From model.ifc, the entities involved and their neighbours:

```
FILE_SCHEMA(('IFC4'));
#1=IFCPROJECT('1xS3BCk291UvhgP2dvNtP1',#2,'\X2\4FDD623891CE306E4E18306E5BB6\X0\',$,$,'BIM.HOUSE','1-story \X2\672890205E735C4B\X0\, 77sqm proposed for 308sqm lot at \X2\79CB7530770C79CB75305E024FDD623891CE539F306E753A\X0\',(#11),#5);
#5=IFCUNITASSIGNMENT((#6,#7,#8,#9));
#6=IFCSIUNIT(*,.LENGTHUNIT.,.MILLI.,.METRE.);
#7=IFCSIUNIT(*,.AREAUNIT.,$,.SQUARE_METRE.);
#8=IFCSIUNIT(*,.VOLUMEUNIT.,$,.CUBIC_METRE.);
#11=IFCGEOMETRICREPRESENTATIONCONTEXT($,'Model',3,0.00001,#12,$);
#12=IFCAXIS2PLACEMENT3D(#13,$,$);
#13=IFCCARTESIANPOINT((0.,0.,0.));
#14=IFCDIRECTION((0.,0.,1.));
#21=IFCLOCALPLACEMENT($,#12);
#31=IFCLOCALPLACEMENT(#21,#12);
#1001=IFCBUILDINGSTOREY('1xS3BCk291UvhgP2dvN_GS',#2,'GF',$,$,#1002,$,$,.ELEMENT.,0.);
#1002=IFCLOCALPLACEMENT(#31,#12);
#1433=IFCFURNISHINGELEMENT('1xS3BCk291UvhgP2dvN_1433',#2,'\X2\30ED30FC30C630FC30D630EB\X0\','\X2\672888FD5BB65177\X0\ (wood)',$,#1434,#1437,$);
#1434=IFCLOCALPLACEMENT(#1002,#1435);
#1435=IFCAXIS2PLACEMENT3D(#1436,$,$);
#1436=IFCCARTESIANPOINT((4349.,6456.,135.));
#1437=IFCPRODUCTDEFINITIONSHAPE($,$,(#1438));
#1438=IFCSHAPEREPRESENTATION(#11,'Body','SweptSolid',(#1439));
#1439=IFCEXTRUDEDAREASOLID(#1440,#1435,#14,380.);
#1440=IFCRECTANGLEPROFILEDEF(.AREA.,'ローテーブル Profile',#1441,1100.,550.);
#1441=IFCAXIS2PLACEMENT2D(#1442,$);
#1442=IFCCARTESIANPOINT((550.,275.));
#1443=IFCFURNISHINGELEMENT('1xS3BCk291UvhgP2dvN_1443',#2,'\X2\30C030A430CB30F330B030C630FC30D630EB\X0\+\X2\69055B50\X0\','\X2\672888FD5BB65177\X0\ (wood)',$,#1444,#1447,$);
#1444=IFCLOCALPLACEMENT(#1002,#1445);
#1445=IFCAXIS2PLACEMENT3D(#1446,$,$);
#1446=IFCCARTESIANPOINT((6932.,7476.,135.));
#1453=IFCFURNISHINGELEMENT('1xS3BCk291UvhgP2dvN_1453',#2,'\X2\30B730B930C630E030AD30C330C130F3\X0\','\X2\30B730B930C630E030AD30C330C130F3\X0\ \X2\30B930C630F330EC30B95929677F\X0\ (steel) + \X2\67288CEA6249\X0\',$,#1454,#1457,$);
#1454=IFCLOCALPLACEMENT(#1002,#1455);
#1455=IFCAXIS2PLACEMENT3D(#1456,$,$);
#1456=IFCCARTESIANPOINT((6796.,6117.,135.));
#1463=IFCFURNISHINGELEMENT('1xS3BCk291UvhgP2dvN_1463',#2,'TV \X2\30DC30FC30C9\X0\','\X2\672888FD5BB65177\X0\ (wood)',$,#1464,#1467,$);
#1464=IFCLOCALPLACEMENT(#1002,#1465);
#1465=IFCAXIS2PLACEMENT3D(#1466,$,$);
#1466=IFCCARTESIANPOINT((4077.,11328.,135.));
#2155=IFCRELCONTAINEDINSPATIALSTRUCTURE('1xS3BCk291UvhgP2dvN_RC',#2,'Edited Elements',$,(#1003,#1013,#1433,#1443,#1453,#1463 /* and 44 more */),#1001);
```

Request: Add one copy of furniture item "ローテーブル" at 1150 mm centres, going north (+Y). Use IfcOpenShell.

```python
import numpy as np
import ifcopenshell
import ifcopenshell.api.geometry
import ifcopenshell.api.root
import ifcopenshell.util.element
import ifcopenshell.util.placement
import ifcopenshell.util.unit

model = ifcopenshell.open("model.ifc")
unit_scale = ifcopenshell.util.unit.calculate_unit_scale(model)


def reuse_history(source, copy):
    """copy_class also copies each property set's owner history, people and application; keep the originals."""
    for rel in copy.IsDefinedBy:
        if rel.is_a("IfcRelDefinesByProperties") and (history := rel.RelatingPropertyDefinition.OwnerHistory):
            rel.RelatingPropertyDefinition.OwnerHistory = source.OwnerHistory
            ifcopenshell.util.element.remove_deep2(model, history)


source = model.by_guid("1xS3BCk291UvhgP2dvN_1433")
base = ifcopenshell.util.placement.get_local_placement(source.ObjectPlacement)
step = np.array([0.0, 1.0, 0.0]) * 1.15 / unit_scale

for i in range(1, 2):
    copy = ifcopenshell.api.root.copy_class(model, product=source)
    copy.Representation = ifcopenshell.util.element.copy_deep(
        model, source.Representation, exclude=["IfcGeometricRepresentationContext", "IfcRepresentationMap"]
    )
    reuse_history(source, copy)
    matrix = base.copy()
    matrix[:3, 3] += i * step
    print("added at", matrix[:3, 3].round(3) + 0.0)
    ifcopenshell.api.geometry.edit_object_placement(model, product=copy, matrix=matrix, is_si=False)

model.write("model_edited.ifc")
```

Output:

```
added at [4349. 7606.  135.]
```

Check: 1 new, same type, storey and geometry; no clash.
